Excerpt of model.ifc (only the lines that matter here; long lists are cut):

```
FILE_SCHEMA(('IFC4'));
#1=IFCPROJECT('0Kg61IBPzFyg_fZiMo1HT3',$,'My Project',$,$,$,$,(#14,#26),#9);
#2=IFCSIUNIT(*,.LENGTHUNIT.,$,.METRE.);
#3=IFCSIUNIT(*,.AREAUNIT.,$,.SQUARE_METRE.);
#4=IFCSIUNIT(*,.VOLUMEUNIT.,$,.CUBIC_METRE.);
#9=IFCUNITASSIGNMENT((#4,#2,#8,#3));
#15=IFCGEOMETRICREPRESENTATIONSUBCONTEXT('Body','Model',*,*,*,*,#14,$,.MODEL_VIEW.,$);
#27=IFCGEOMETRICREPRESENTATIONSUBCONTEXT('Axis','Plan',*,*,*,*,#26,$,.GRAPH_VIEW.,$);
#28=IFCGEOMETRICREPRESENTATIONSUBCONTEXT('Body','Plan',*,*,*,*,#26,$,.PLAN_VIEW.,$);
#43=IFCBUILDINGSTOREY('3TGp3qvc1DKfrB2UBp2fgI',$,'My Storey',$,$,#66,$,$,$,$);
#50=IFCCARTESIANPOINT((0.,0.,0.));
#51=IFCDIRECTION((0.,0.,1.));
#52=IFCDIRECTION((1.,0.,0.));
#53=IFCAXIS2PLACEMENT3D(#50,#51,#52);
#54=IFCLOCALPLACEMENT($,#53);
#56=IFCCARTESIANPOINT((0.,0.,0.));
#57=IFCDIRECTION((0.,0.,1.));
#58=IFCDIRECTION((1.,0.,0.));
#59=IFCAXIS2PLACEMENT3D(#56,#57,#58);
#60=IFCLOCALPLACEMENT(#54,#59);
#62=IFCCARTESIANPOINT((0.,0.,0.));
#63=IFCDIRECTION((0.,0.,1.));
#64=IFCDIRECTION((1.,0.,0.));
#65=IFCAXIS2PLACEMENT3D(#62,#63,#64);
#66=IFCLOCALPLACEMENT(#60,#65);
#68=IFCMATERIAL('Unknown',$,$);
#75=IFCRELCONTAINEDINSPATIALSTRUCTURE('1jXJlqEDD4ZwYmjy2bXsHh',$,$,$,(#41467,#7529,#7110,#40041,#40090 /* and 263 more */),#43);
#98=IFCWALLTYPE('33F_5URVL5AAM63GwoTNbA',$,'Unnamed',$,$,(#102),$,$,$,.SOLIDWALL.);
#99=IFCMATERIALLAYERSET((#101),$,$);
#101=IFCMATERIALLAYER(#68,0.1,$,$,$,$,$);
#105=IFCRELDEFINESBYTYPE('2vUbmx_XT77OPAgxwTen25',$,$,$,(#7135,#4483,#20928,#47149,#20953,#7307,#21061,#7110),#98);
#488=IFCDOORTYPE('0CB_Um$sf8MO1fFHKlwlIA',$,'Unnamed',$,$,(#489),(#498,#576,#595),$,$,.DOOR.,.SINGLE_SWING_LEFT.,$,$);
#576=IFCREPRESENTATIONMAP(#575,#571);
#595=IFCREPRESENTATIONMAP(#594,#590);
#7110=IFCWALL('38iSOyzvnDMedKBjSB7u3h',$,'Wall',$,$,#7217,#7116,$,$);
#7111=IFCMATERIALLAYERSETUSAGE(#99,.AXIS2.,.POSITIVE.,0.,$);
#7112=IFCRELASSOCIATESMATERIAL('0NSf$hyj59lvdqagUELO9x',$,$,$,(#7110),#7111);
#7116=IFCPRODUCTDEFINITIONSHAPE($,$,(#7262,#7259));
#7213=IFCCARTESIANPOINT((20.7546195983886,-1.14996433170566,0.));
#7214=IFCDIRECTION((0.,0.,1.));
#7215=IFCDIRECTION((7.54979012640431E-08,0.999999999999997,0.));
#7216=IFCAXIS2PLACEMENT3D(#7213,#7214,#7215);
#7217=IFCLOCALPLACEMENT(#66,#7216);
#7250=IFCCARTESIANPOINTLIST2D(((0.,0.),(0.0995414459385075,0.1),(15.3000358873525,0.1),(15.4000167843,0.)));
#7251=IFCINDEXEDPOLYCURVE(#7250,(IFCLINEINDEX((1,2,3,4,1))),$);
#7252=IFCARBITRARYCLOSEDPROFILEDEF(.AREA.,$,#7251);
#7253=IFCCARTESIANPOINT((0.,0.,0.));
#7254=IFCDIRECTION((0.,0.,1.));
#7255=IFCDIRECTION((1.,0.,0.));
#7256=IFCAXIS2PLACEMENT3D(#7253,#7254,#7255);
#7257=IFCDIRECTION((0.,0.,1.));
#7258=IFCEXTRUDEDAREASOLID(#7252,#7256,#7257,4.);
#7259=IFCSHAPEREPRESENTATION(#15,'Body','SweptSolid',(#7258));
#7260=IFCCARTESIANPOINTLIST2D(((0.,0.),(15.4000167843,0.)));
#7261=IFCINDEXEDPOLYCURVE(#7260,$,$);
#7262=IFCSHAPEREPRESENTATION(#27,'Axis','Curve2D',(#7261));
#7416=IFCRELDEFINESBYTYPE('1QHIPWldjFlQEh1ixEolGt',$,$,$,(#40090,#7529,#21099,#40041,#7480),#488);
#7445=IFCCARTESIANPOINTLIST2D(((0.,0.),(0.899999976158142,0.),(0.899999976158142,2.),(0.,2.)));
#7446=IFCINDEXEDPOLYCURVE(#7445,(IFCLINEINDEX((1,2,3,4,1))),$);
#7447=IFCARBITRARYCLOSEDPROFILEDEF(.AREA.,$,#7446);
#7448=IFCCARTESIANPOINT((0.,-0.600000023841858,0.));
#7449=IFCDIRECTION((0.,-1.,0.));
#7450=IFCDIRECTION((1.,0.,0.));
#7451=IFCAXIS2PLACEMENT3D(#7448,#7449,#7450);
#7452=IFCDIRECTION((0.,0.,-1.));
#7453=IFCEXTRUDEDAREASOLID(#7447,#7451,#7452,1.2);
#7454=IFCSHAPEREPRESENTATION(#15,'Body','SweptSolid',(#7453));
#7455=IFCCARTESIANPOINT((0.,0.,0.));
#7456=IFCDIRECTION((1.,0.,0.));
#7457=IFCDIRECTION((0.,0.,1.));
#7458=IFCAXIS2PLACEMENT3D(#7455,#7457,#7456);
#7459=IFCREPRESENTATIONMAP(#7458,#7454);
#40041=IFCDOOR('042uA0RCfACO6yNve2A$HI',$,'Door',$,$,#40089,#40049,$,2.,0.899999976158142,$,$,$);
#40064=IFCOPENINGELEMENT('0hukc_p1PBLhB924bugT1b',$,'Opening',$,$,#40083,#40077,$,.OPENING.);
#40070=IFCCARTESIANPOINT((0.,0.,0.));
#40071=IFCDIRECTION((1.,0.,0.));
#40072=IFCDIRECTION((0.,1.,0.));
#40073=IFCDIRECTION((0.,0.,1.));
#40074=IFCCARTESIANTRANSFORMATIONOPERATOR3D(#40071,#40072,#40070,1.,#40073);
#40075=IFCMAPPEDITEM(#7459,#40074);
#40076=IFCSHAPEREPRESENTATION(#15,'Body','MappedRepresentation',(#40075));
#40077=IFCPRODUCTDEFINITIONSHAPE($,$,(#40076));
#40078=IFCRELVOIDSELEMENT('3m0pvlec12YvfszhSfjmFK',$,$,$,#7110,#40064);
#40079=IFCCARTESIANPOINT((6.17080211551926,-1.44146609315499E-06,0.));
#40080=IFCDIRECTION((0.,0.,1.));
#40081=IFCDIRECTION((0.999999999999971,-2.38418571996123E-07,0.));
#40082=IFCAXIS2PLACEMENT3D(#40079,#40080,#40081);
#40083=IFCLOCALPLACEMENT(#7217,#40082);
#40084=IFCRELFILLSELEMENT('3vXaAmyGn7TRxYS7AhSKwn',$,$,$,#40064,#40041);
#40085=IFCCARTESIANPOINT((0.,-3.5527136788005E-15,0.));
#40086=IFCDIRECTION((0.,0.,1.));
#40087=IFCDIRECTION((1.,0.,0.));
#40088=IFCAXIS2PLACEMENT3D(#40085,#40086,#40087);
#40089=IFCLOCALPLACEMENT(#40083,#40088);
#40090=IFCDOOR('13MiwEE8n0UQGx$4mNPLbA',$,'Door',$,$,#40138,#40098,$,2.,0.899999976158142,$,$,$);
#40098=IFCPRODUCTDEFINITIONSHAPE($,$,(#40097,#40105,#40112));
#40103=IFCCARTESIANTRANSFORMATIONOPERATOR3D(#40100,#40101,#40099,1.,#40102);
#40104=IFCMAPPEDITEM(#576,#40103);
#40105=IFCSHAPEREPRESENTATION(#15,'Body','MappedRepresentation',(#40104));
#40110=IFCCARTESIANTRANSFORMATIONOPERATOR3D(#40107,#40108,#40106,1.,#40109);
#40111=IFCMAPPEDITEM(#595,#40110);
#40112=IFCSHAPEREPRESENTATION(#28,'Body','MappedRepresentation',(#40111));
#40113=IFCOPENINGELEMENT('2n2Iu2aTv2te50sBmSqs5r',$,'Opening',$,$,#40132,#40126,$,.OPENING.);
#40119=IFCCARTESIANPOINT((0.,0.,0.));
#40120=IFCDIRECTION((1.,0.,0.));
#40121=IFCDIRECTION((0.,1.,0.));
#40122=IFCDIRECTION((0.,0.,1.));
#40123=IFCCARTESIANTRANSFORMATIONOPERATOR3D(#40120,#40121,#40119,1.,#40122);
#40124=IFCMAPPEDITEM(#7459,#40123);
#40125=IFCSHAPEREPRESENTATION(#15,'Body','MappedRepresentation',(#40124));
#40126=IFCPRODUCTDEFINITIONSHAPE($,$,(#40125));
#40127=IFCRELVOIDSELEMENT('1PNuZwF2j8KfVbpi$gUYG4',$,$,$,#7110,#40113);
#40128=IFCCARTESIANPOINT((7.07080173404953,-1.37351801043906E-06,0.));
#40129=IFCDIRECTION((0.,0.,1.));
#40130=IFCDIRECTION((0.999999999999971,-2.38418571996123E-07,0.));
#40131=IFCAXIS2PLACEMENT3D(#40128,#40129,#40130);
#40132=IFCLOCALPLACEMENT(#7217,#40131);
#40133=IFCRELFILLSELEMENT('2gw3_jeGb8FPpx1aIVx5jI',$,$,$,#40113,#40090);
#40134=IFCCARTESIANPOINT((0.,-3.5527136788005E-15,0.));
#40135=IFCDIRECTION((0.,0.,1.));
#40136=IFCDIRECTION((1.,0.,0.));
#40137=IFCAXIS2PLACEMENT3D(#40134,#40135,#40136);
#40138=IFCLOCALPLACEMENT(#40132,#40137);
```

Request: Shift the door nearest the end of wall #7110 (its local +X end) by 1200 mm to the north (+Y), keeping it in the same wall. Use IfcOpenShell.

```python
import ifcopenshell
import ifcopenshell.api.geometry
import ifcopenshell.util.placement
import ifcopenshell.util.unit

model = ifcopenshell.open("model.ifc")
unit_scale = ifcopenshell.util.unit.calculate_unit_scale(model)

door = model.by_id(40090)
opening = door.FillsVoids[0].RelatingOpeningElement
wall = opening.VoidsElements[0].RelatingBuildingElement

wall_matrix = ifcopenshell.util.placement.get_local_placement(wall.ObjectPlacement)
shift = wall_matrix[:3, 0] * 1.2 / unit_scale
before = ifcopenshell.util.placement.get_local_placement(door.ObjectPlacement)[:3, 3].copy()

# The door is placed relative to its opening, so it follows when the opening moves.
matrix = ifcopenshell.util.placement.get_local_placement(opening.ObjectPlacement)
matrix[:3, 3] += shift
ifcopenshell.api.geometry.edit_object_placement(
    model, product=opening, matrix=matrix, is_si=False, should_transform_children=True
)

after = ifcopenshell.util.placement.get_local_placement(door.ObjectPlacement)[:3, 3]
print("door moved by", (after - before).round(3) + 0.0)

model.write("model_rev.ifc")
```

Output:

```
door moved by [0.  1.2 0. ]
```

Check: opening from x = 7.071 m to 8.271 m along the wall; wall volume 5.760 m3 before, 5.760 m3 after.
